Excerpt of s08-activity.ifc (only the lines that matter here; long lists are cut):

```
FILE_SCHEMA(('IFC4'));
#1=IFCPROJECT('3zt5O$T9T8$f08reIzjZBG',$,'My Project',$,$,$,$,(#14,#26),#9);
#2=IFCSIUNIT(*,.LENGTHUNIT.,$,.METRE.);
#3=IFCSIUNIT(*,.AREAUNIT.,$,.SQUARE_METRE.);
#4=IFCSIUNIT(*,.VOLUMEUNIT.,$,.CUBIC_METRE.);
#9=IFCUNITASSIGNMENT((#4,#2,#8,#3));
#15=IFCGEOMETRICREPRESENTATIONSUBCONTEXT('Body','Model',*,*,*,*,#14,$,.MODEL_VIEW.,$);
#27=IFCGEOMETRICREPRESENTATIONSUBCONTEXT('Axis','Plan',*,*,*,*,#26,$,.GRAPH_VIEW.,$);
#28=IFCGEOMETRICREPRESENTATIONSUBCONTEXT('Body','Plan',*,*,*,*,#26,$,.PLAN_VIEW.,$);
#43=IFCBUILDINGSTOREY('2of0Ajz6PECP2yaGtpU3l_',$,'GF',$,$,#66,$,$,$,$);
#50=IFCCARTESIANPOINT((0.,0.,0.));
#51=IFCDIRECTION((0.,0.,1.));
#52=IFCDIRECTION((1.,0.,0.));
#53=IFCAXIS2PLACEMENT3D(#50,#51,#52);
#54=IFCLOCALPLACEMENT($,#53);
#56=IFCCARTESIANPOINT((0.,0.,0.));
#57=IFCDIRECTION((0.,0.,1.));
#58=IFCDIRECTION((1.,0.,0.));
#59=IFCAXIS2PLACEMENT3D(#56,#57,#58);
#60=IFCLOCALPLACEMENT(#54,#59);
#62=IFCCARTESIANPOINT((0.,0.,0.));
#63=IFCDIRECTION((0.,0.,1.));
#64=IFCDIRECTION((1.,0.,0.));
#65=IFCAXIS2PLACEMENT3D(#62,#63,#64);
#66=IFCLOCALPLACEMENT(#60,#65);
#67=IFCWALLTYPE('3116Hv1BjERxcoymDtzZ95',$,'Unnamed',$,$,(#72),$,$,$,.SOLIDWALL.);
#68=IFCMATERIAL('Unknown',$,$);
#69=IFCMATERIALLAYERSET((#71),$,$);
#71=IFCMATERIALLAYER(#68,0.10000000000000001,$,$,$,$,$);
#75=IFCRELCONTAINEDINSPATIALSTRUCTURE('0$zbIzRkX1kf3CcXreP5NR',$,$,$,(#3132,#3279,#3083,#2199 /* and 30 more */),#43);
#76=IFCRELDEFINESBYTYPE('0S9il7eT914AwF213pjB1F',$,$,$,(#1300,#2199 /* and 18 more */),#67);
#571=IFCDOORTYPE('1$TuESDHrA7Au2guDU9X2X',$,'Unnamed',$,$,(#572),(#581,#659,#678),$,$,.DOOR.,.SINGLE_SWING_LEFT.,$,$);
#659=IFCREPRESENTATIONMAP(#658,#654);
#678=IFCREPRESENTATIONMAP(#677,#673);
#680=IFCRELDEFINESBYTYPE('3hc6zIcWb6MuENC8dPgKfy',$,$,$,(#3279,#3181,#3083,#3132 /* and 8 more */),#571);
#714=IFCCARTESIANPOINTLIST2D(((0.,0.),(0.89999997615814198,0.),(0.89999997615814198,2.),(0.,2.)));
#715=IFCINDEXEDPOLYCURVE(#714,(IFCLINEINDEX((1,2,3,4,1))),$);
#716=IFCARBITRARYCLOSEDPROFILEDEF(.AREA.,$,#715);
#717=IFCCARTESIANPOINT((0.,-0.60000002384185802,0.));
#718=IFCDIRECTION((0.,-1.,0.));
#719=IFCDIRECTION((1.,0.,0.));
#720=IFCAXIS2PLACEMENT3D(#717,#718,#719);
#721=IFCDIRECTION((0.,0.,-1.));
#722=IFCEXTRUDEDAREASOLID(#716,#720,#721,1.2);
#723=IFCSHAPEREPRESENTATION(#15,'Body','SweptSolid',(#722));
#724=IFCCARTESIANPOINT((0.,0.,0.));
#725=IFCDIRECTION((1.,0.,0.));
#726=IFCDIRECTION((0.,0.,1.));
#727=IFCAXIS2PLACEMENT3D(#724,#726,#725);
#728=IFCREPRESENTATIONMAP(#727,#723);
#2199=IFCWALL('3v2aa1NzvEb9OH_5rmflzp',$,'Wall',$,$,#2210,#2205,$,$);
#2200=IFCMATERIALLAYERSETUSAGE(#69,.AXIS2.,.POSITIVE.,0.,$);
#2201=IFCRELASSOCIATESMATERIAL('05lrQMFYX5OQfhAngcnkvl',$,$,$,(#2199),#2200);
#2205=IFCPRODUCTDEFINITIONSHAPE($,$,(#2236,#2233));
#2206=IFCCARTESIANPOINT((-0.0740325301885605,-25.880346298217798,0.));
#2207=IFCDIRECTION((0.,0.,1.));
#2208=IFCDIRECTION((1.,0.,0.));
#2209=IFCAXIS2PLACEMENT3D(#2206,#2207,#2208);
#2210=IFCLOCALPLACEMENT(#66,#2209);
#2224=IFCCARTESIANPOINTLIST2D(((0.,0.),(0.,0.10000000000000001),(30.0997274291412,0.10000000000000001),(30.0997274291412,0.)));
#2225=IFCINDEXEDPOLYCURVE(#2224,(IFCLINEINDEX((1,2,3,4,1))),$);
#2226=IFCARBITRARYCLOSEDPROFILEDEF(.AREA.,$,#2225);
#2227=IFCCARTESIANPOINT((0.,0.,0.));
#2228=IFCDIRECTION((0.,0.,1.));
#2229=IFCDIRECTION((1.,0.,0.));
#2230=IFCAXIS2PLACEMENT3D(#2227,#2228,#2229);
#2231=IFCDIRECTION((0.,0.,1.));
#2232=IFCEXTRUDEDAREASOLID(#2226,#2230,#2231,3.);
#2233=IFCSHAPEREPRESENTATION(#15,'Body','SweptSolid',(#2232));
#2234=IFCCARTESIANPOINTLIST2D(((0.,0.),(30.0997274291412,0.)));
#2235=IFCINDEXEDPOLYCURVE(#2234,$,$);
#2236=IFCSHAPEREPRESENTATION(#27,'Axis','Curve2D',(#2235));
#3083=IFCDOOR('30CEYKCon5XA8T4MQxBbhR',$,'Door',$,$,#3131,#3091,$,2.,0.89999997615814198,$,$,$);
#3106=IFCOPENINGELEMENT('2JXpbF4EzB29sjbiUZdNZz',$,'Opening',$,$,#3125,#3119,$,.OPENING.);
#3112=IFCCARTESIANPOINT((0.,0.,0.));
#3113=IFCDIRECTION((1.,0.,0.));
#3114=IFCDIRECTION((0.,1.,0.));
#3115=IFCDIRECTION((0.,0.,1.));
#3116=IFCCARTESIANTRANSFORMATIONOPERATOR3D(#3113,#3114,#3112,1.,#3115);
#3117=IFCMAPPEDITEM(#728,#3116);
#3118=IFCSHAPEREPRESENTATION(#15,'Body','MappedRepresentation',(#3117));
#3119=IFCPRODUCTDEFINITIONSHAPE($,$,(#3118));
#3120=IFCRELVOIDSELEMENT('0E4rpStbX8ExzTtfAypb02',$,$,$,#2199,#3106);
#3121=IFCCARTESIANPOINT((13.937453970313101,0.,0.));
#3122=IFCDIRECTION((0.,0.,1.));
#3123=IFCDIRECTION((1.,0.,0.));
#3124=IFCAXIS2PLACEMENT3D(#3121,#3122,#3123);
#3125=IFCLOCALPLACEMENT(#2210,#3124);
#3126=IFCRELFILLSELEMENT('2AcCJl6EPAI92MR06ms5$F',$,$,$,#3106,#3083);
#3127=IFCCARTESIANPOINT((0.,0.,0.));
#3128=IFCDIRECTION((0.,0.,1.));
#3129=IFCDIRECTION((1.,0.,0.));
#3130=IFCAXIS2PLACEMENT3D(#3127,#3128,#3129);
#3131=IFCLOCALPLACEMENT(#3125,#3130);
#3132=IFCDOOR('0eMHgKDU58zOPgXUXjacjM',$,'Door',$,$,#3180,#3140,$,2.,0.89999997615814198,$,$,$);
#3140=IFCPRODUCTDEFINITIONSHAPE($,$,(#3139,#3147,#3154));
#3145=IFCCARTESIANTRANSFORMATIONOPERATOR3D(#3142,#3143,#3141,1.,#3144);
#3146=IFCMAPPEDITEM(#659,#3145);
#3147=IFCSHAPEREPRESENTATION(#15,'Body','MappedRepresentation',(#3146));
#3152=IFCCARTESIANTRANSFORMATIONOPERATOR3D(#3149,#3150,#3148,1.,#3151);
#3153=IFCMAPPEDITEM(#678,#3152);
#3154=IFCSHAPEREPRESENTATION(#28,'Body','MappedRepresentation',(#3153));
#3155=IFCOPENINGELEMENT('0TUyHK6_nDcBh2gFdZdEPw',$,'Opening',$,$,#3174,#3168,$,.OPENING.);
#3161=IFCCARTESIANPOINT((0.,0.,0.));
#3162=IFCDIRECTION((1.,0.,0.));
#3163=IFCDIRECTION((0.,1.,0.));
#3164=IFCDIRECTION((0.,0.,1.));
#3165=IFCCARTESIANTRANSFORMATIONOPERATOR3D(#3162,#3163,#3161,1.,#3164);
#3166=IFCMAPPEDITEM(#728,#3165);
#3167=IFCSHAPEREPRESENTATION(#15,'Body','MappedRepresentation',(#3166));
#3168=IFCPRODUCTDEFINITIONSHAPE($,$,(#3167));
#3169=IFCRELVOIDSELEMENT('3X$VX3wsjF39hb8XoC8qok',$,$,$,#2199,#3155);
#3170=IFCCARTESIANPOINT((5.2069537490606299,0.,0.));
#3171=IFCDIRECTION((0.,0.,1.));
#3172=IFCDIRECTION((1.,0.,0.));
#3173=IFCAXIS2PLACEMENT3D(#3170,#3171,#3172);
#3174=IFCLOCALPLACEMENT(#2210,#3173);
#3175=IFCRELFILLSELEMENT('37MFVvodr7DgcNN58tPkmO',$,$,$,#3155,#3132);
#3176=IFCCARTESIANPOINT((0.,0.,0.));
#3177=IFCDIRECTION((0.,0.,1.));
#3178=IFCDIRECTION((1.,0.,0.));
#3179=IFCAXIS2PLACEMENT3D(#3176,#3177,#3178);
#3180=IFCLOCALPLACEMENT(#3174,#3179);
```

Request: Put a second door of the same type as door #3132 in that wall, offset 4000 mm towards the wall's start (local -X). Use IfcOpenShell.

```python
import ifcopenshell
import ifcopenshell.api.feature
import ifcopenshell.api.geometry
import ifcopenshell.api.root
import ifcopenshell.geom
import ifcopenshell.util.element
import ifcopenshell.util.placement
import ifcopenshell.util.shape
import ifcopenshell.util.unit

model = ifcopenshell.open("s08-activity.ifc")
unit_scale = ifcopenshell.util.unit.calculate_unit_scale(model)
settings = ifcopenshell.geom.settings()


def volume(element):
    """Net volume in cubic metres, openings subtracted."""
    shape = ifcopenshell.geom.create_shape(settings, element)
    return ifcopenshell.util.shape.get_volume(shape.geometry)


door = model.by_guid("0eMHgKDU58zOPgXUXjacjM")
opening = door.FillsVoids[0].RelatingOpeningElement
wall = opening.VoidsElements[0].RelatingBuildingElement
before = volume(wall)
shift = ifcopenshell.util.placement.get_local_placement(wall.ObjectPlacement)[:3, 0] * -4 / unit_scale

# copy_class copies the void relationship, type, container and properties, but no geometry.
new_opening = ifcopenshell.api.root.copy_class(model, product=opening)
new_opening.Representation = ifcopenshell.util.element.copy_deep(
    model, opening.Representation, exclude=["IfcGeometricRepresentationContext", "IfcRepresentationMap"]
)
new_door = ifcopenshell.api.root.copy_class(model, product=door)
new_door.Representation = ifcopenshell.util.element.copy_deep(
    model, door.Representation, exclude=["IfcGeometricRepresentationContext", "IfcRepresentationMap"]
)
ifcopenshell.api.feature.add_filling(model, opening=new_opening, element=new_door)

for old, new in ((opening, new_opening), (door, new_door)):
    matrix = ifcopenshell.util.placement.get_local_placement(old.ObjectPlacement)
    matrix[:3, 3] += shift
    ifcopenshell.api.geometry.edit_object_placement(model, product=new, matrix=matrix, is_si=False)

after = volume(wall)

print(f"wall volume {before:.3f} -> {after:.3f} m3")

model.write("s08-activity_v2.ifc")
```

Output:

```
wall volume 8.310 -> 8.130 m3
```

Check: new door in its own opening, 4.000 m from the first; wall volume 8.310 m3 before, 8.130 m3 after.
